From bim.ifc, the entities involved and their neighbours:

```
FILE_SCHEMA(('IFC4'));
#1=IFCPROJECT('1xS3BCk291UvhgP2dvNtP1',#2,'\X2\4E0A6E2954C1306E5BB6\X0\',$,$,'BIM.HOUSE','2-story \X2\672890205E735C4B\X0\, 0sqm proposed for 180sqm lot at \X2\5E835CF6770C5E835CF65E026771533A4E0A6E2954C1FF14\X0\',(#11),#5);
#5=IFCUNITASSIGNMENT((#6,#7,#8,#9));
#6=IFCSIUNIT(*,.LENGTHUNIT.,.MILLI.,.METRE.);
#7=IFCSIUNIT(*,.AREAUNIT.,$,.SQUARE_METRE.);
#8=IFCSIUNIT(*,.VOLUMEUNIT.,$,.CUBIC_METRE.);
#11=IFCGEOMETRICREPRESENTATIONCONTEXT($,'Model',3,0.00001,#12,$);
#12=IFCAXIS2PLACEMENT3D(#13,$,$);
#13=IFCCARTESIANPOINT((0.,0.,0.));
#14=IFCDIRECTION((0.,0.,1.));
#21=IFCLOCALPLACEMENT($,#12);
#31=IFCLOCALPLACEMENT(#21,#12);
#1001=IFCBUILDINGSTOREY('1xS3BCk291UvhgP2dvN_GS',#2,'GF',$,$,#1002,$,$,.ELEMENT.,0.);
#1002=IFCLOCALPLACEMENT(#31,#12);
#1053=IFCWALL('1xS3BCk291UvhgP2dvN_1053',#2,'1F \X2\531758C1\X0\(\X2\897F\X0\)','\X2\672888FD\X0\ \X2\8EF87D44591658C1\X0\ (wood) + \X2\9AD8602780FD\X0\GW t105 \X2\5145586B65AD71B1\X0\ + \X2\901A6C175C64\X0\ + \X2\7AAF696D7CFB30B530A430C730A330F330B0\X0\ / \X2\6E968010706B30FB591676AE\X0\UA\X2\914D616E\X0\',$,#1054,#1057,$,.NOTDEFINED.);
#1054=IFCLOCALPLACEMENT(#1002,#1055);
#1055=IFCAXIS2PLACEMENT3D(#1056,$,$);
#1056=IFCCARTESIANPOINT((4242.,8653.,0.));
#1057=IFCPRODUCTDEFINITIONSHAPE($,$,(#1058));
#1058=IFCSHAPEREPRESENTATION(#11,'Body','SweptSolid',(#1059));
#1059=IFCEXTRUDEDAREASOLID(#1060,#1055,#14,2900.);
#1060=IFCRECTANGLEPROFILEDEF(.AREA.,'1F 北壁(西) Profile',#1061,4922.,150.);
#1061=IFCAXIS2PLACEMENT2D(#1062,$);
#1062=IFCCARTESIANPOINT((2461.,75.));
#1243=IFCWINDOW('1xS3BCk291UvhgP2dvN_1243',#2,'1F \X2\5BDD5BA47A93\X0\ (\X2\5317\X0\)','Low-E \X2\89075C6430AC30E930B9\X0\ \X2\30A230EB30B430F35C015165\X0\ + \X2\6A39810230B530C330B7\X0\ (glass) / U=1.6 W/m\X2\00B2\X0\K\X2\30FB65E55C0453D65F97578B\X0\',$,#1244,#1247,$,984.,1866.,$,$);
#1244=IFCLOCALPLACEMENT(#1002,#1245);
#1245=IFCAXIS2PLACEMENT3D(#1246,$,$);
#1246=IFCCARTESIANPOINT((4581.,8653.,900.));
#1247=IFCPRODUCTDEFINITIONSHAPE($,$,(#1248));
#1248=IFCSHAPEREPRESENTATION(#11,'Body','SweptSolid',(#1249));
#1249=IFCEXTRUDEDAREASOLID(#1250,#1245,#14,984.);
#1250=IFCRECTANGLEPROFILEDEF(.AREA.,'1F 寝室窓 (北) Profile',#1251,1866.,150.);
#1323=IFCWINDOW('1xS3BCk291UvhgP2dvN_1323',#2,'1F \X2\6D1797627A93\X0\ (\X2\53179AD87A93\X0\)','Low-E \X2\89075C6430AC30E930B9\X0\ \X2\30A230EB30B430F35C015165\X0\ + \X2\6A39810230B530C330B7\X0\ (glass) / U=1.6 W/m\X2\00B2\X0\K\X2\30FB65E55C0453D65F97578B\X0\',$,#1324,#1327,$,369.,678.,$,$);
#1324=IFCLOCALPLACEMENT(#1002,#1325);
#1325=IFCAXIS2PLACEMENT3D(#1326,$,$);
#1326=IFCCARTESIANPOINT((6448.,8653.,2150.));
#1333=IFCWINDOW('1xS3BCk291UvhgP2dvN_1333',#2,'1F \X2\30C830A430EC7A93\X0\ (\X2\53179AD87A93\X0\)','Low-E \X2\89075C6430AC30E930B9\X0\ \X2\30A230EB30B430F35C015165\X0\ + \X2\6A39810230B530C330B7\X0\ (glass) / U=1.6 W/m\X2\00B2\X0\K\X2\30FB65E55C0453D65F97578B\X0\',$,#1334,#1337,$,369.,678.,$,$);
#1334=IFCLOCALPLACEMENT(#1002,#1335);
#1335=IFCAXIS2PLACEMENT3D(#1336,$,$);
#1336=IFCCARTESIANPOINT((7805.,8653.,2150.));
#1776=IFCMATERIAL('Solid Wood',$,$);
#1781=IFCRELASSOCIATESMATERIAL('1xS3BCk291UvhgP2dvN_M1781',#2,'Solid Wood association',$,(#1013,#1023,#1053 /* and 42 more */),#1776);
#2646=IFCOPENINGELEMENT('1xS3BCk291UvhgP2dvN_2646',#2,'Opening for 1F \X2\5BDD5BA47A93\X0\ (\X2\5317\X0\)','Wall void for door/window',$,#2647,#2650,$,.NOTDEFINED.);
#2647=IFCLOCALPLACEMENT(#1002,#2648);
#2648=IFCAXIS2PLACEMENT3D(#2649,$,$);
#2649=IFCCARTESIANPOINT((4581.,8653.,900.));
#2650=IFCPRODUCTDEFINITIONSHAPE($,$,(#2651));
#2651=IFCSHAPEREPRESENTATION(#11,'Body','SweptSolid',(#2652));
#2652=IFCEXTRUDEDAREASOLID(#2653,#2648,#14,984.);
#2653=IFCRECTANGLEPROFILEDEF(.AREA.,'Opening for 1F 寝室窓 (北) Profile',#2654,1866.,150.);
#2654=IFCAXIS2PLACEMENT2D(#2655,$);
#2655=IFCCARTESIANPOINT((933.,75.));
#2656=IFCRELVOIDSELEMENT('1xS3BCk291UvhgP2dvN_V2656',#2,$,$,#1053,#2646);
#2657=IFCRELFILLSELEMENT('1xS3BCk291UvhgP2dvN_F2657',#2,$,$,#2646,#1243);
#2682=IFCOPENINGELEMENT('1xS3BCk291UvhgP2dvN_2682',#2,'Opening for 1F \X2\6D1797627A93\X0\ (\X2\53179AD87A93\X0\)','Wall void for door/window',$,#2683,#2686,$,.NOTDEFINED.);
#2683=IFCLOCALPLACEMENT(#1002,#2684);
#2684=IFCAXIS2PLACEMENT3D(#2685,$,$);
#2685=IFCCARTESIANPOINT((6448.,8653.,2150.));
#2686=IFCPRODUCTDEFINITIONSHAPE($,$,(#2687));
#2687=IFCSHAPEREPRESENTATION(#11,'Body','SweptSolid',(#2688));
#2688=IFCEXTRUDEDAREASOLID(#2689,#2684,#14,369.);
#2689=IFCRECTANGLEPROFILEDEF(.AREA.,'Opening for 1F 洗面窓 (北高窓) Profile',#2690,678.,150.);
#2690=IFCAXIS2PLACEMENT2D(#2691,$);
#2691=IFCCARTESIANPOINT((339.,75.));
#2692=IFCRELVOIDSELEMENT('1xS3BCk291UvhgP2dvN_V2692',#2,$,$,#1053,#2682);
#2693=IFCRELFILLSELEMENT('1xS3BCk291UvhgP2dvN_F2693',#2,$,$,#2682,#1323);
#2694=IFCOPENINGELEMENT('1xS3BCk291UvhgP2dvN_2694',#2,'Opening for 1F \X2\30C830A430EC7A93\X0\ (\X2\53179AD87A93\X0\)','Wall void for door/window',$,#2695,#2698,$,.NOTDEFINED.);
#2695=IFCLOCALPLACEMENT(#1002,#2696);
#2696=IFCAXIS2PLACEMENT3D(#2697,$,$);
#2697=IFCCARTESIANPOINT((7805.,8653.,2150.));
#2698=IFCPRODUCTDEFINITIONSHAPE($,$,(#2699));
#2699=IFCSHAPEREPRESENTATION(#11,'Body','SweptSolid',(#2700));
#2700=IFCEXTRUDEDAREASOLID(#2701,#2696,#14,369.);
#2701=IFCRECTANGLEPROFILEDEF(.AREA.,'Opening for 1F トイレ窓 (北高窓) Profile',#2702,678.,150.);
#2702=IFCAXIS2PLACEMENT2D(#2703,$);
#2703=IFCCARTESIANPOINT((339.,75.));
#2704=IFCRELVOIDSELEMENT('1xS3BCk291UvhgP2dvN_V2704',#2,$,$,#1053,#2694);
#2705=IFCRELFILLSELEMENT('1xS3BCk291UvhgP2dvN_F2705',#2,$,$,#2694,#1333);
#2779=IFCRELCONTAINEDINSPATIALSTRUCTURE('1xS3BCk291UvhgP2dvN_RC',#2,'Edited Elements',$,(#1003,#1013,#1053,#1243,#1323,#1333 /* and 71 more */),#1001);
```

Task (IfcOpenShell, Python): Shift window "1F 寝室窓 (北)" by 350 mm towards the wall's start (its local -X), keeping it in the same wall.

```python
import ifcopenshell
import ifcopenshell.api.geometry
import ifcopenshell.util.placement
import ifcopenshell.util.unit

model = ifcopenshell.open("bim.ifc")
unit_scale = ifcopenshell.util.unit.calculate_unit_scale(model)

window = model.by_guid("1xS3BCk291UvhgP2dvN_1243")
opening = window.FillsVoids[0].RelatingOpeningElement
wall = opening.VoidsElements[0].RelatingBuildingElement

wall_matrix = ifcopenshell.util.placement.get_local_placement(wall.ObjectPlacement)
shift = wall_matrix[:3, 0] * -0.35 / unit_scale
before = ifcopenshell.util.placement.get_local_placement(window.ObjectPlacement)[:3, 3].copy()

# The window is not placed relative to its opening, so move both.
for product in (opening, window):
    matrix = ifcopenshell.util.placement.get_local_placement(product.ObjectPlacement)
    matrix[:3, 3] += shift
    ifcopenshell.api.geometry.edit_object_placement(model, product=product, matrix=matrix, is_si=False)

after = ifcopenshell.util.placement.get_local_placement(window.ObjectPlacement)[:3, 3]
print("window moved by", (after - before).round(3) + 0.0)

model.write("bim_updated.ifc")
```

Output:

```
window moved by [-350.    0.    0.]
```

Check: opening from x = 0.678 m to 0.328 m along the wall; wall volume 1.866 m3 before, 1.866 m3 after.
